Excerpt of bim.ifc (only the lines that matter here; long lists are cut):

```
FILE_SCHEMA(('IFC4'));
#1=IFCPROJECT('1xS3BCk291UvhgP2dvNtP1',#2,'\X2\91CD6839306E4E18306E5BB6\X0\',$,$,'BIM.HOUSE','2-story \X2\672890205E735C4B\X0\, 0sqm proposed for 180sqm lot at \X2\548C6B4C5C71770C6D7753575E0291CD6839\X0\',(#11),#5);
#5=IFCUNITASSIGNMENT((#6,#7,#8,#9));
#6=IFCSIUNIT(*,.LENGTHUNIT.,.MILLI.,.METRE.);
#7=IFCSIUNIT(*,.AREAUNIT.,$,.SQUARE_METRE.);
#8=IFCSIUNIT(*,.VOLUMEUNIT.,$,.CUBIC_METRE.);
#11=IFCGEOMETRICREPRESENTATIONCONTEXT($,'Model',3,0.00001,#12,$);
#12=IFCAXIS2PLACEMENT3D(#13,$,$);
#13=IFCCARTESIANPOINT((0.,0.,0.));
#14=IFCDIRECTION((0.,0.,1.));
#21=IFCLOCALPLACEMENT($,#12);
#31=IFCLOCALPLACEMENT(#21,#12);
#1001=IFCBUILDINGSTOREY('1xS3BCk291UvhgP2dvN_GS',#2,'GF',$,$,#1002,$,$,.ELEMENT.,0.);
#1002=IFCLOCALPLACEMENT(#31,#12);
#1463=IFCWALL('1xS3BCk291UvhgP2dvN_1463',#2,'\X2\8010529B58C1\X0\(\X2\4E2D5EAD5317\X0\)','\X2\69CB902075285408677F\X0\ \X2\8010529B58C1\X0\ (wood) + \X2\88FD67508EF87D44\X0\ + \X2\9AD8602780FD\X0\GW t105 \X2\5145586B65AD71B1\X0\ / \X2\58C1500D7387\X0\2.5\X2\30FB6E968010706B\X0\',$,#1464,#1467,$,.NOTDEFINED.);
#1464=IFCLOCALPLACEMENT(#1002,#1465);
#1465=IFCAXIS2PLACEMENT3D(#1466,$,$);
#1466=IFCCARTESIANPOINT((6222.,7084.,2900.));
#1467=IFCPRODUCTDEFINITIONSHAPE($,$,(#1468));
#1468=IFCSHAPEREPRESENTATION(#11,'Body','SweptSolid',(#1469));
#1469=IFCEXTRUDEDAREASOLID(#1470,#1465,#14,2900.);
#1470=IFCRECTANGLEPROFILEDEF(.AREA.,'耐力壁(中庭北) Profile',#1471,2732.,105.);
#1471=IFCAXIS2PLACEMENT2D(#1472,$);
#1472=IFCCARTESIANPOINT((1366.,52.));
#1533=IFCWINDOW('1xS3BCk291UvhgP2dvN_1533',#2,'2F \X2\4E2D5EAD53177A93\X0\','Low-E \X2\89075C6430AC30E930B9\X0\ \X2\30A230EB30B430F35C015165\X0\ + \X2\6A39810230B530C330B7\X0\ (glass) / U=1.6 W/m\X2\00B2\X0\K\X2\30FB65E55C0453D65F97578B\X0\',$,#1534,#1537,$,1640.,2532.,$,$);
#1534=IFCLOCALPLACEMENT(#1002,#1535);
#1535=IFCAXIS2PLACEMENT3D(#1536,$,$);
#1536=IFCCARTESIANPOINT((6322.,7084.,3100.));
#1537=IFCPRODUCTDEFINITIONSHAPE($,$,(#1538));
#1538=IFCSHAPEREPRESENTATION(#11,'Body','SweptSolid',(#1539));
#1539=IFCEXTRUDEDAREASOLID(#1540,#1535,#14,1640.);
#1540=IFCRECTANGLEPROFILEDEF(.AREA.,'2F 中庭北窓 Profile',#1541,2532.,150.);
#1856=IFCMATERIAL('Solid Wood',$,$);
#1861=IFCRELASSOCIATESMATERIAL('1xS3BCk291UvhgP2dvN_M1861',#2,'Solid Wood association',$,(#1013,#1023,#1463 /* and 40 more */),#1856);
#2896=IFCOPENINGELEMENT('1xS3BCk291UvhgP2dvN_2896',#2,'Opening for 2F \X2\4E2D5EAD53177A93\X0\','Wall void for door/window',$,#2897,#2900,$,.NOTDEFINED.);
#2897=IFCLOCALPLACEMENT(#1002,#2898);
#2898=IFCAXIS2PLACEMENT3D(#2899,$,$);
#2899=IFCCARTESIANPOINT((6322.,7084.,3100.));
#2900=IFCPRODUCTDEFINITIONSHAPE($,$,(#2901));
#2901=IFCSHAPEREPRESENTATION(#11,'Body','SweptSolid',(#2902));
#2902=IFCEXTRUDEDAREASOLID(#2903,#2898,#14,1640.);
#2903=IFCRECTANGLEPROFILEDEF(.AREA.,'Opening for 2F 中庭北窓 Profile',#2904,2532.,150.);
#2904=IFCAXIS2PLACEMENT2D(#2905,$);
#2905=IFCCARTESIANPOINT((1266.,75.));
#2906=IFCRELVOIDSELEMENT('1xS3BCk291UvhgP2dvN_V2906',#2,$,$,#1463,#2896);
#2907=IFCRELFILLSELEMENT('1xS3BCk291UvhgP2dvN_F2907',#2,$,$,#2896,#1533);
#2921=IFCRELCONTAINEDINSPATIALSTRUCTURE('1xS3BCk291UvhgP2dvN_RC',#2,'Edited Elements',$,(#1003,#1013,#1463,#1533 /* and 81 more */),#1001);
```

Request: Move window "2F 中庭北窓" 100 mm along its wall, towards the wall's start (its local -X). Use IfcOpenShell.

```python
import ifcopenshell
import ifcopenshell.api.geometry
import ifcopenshell.util.placement
import ifcopenshell.util.unit

model = ifcopenshell.open("bim.ifc")
unit_scale = ifcopenshell.util.unit.calculate_unit_scale(model)

window = model.by_id(1533)
opening = window.FillsVoids[0].RelatingOpeningElement
wall = opening.VoidsElements[0].RelatingBuildingElement

wall_matrix = ifcopenshell.util.placement.get_local_placement(wall.ObjectPlacement)
shift = wall_matrix[:3, 0] * -0.1 / unit_scale
before = ifcopenshell.util.placement.get_local_placement(window.ObjectPlacement)[:3, 3].copy()

# The window is not placed relative to its opening, so move both.
for product in (opening, window):
    matrix = ifcopenshell.util.placement.get_local_placement(product.ObjectPlacement)
    matrix[:3, 3] += shift
    ifcopenshell.api.geometry.edit_object_placement(model, product=product, matrix=matrix, is_si=False)

after = ifcopenshell.util.placement.get_local_placement(window.ObjectPlacement)[:3, 3]
print("window moved by", (after - before).round(3) + 0.0)

model.write("bim_updated.ifc")
```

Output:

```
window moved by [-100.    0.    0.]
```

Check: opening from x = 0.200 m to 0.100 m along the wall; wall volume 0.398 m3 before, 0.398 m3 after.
